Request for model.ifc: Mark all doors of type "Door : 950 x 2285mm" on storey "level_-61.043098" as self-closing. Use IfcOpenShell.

First a look at what the model holds.

```python
import ifcopenshell
import ifcopenshell.util.element

model = ifcopenshell.open("model.ifc")
print(model.schema)
storey = next(s for s in model.by_type("IfcBuildingStorey") if s.Name == "level_-61.043098")
doors = [e for e in ifcopenshell.util.element.get_decomposition(storey) if e.is_a("IfcDoor")]
seen = {}
for e in doors:
    element_type = ifcopenshell.util.element.get_type(e)
    key = (element_type.Name if element_type != e and element_type else None, ifcopenshell.util.element.get_pset(e, "Pset_DoorCommon", "SelfClosing"))
    seen[key] = seen.get(key, 0) + 1
for (name, value), count in sorted(seen.items(), key=str):
    print(count, "x", name, "|", value)
```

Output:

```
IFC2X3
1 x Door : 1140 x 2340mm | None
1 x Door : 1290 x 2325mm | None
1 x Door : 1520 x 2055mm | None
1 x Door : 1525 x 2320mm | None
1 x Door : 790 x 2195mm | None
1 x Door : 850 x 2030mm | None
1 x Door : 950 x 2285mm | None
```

```python
import ifcopenshell
import ifcopenshell.api.pset
import ifcopenshell.util.element

model = ifcopenshell.open("model.ifc")

storey = next(s for s in model.by_type("IfcBuildingStorey") if s.Name == "level_-61.043098")
doors = [e for e in ifcopenshell.util.element.get_decomposition(storey) if e.is_a("IfcDoor")]

count = 0
for e in doors:
    element_type = ifcopenshell.util.element.get_type(e)
    if element_type in (None, e) or element_type.Name != "Door : 950 x 2285mm":
        continue
    # add_pset returns the element's existing set when there is one.
    pset = ifcopenshell.api.pset.add_pset(model, product=e, name="Pset_DoorCommon")
    ifcopenshell.api.pset.edit_pset(model, pset=pset, properties={"SelfClosing": True})
    count += 1

print(count, "doors updated")

model.write("model_edited.ifc")
```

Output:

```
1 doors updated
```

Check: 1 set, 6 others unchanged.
